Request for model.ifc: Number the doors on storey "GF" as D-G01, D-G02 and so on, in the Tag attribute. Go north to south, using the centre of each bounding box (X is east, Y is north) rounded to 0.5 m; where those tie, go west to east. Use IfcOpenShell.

First a look at what the model holds.

```python
import ifcopenshell
import ifcopenshell.util.element
import ifcopenshell.util.placement

model = ifcopenshell.open("model.ifc")
print(model.schema)
storey = next(s for s in model.by_type("IfcBuildingStorey") if s.Name == "GF")
doors = [e for e in ifcopenshell.util.element.get_decomposition(storey) if e.is_a("IfcDoor")]
for e in sorted(doors, key=lambda e: e.id()):
    origin = ifcopenshell.util.placement.get_local_placement(e.ObjectPlacement)[:3, 3]
    print(e.id(), e.Tag, e.Name, origin.round(2) + 0.0, sep=" | ")
```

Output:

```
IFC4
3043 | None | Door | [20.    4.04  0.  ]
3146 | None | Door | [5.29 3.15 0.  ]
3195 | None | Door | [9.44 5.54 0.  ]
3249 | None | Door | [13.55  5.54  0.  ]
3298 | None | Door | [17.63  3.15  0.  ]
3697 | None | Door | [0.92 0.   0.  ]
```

```python
import ifcopenshell
import ifcopenshell.geom
import ifcopenshell.util.element
import ifcopenshell.util.shape

model = ifcopenshell.open("model.ifc")
settings = ifcopenshell.geom.settings()
settings.set("use-world-coords", True)


def centre(element):
    shape = ifcopenshell.geom.create_shape(settings, element)
    return ifcopenshell.util.shape.get_bbox_centroid(shape.geometry)


storey = next(s for s in model.by_type("IfcBuildingStorey") if s.Name == "GF")
doors = [e for e in ifcopenshell.util.element.get_decomposition(storey) if e.is_a("IfcDoor")]

# Insertion points can sit at a corner or the storey origin, so sort by the geometry (in metres).
centres = {e: centre(e) for e in doors}
doors.sort(key=lambda e: (-round(centres[e][1] / 0.5), centres[e][0]))

for i, e in enumerate(doors, start=1):
    number = f"D-G{i:02d}"
    e.Tag = number
    print(e.id(), number)

model.write("model-out.ifc")
```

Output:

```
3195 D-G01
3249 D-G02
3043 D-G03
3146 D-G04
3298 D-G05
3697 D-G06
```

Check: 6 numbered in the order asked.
